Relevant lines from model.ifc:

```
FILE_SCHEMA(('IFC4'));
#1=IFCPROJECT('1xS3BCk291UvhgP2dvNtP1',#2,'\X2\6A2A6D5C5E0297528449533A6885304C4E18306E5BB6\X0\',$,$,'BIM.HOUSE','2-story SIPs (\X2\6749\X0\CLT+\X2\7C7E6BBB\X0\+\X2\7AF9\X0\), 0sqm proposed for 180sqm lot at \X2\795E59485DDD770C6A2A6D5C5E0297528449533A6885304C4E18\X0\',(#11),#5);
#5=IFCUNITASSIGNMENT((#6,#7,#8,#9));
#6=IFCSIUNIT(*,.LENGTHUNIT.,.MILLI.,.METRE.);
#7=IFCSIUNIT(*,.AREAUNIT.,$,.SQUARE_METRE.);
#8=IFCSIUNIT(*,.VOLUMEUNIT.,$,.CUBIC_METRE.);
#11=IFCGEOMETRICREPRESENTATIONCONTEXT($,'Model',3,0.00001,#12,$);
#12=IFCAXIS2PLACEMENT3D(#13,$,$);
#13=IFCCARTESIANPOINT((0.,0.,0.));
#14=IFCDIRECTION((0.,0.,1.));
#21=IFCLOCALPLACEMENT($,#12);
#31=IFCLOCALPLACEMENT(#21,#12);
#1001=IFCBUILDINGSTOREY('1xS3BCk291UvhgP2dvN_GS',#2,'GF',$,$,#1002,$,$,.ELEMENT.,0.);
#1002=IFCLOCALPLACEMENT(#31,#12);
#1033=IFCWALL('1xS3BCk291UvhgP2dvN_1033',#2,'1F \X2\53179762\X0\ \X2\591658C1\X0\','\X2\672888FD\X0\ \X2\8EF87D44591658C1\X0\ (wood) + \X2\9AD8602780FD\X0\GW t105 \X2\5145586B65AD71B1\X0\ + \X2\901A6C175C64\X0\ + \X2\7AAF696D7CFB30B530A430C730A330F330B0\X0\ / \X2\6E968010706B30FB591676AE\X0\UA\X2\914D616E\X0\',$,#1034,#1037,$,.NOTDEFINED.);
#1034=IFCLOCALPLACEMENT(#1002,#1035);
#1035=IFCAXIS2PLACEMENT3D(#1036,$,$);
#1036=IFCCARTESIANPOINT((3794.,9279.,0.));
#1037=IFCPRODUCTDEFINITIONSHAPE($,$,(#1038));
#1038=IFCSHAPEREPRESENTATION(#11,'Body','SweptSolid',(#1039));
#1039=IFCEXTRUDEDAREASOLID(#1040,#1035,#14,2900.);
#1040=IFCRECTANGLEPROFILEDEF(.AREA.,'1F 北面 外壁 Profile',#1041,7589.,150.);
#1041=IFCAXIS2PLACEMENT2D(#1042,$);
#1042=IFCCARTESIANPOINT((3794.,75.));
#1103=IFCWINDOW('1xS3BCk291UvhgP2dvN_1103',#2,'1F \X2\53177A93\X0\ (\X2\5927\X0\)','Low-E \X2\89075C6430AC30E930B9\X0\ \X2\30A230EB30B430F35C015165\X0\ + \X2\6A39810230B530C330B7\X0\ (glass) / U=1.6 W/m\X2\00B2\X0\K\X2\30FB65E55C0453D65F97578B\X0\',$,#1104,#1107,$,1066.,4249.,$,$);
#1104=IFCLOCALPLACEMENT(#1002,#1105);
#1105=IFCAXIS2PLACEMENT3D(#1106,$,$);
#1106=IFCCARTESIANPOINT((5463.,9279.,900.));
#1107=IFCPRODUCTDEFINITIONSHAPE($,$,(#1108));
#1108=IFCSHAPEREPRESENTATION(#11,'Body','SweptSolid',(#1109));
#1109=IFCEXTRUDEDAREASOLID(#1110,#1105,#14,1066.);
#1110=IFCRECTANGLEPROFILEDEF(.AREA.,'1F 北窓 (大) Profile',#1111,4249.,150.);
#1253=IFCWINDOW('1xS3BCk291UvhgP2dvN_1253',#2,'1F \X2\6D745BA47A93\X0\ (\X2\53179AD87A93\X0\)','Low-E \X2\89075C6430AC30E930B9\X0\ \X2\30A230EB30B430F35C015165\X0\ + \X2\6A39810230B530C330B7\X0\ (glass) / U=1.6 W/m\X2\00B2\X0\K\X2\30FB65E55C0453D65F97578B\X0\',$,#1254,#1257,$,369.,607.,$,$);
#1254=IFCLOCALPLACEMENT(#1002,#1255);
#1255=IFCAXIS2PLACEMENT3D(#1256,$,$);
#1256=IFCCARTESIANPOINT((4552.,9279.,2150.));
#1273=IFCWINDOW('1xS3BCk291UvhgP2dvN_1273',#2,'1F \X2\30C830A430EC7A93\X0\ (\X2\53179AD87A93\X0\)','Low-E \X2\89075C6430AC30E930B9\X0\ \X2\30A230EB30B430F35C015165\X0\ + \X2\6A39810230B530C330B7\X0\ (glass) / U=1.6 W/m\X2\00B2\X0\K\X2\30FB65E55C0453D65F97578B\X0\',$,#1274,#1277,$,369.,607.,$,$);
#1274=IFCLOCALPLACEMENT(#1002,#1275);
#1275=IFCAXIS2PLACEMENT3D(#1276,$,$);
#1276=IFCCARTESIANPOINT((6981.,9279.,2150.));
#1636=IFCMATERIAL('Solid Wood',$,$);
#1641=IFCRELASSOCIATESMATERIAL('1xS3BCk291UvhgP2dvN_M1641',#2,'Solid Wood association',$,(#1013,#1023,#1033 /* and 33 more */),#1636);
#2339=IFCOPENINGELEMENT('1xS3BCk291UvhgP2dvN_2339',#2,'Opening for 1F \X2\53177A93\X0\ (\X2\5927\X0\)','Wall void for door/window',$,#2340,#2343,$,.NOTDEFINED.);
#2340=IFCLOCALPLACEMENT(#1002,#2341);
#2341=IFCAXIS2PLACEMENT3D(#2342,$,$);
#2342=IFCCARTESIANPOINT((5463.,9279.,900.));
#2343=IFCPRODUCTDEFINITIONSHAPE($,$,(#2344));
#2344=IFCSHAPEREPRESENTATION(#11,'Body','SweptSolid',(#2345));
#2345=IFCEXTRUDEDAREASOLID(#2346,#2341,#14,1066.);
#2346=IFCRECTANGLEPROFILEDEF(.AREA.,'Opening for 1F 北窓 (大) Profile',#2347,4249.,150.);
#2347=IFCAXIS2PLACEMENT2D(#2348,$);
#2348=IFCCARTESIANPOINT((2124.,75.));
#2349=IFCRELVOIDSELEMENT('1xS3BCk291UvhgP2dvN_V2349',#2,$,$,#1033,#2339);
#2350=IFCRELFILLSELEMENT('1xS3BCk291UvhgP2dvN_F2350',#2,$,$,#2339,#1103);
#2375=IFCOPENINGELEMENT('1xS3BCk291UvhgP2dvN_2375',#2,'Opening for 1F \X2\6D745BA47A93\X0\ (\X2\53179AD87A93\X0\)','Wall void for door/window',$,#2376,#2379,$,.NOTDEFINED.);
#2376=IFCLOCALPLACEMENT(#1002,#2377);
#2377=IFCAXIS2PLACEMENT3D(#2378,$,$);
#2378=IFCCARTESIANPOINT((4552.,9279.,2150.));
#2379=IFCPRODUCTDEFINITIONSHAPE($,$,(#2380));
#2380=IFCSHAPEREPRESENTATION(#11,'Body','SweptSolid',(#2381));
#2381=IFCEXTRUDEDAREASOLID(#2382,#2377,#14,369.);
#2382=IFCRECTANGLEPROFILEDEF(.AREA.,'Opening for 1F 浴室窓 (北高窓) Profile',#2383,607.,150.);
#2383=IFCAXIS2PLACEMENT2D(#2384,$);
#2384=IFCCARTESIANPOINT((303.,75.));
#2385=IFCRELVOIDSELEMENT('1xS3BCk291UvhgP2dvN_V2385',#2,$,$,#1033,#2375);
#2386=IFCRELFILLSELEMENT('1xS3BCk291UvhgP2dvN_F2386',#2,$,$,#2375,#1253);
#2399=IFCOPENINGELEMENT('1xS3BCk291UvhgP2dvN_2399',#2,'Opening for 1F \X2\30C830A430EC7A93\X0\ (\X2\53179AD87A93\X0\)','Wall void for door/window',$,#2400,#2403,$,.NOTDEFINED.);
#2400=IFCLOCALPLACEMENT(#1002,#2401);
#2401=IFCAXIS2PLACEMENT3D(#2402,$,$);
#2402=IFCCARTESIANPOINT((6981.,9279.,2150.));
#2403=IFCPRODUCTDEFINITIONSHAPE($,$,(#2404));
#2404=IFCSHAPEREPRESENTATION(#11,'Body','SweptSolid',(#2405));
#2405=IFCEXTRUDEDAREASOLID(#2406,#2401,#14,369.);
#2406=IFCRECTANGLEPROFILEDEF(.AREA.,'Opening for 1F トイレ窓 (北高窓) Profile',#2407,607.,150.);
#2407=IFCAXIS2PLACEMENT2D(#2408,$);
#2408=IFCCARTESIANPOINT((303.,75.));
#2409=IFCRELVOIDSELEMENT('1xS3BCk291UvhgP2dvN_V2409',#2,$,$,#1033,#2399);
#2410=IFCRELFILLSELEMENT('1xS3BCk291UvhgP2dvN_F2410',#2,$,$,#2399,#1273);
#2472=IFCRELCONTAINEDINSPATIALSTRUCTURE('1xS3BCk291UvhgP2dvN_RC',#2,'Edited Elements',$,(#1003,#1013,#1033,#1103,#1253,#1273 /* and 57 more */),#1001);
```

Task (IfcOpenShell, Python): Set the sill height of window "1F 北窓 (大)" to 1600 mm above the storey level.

```python
import numpy as np
import ifcopenshell
import ifcopenshell.api.geometry
import ifcopenshell.geom
import ifcopenshell.util.element
import ifcopenshell.util.placement
import ifcopenshell.util.shape
import ifcopenshell.util.unit

model = ifcopenshell.open("model.ifc")
unit_scale = ifcopenshell.util.unit.calculate_unit_scale(model)

window = model.by_id(1103)
opening = window.FillsVoids[0].RelatingOpeningElement
storey = ifcopenshell.util.element.get_container(window, ifc_class="IfcBuildingStorey")
level = ifcopenshell.util.placement.get_local_placement(storey.ObjectPlacement)[2, 3]

# The opening's origin need not be at the sill, so measure its lowest point.
shape = ifcopenshell.geom.create_shape(ifcopenshell.geom.settings(), opening)
bottom = ifcopenshell.util.shape.get_shape_bottom_elevation(shape, shape.geometry) / unit_scale
dz = level + 1600.0 - bottom

shift = np.array([0.0, 0.0, dz])
# The window is not placed relative to its opening, so move both.
for product in (opening, window):
    matrix = ifcopenshell.util.placement.get_local_placement(product.ObjectPlacement)
    matrix[:3, 3] += shift
    ifcopenshell.api.geometry.edit_object_placement(model, product=product, matrix=matrix, is_si=False)

print(f"moved by {dz * unit_scale:+.3f} m")

model.write("model_edited.ifc")
```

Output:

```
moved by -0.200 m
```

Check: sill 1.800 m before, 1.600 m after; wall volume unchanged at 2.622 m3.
